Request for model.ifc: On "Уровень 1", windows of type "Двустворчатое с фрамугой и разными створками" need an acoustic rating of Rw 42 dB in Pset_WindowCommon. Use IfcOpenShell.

First a look at what the model holds.

```python
import ifcopenshell
import ifcopenshell.util.element

model = ifcopenshell.open("model.ifc")
print(model.schema)
storey = next(s for s in model.by_type("IfcBuildingStorey") if s.Name == "Уровень 1")
windows = [e for e in ifcopenshell.util.element.get_decomposition(storey) if e.is_a("IfcWindow")]
seen = {}
for e in windows:
    element_type = ifcopenshell.util.element.get_type(e)
    key = (element_type.Name if element_type != e and element_type else None, ifcopenshell.util.element.get_pset(e, "Pset_WindowCommon", "AcousticRating"))
    seen[key] = seen.get(key, 0) + 1
for (name, value), count in sorted(seen.items(), key=str):
    print(count, "x", name, "|", value)
```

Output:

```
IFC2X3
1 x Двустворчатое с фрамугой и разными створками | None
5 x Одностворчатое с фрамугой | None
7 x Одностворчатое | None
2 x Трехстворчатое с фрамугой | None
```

```python
import ifcopenshell
import ifcopenshell.api.pset
import ifcopenshell.util.element

model = ifcopenshell.open("model.ifc")

storey = next(s for s in model.by_type("IfcBuildingStorey") if s.Name == "Уровень 1")
windows = [e for e in ifcopenshell.util.element.get_decomposition(storey) if e.is_a("IfcWindow")]

count = 0
for e in windows:
    element_type = ifcopenshell.util.element.get_type(e)
    if element_type in (None, e) or element_type.Name != "Двустворчатое с фрамугой и разными створками":
        continue
    # add_pset returns the element's existing set when there is one.
    pset = ifcopenshell.api.pset.add_pset(model, product=e, name="Pset_WindowCommon")
    ifcopenshell.api.pset.edit_pset(model, pset=pset, properties={"AcousticRating": "Rw 42 dB"})
    count += 1

print(count, "windows updated")

model.write("model_edited.ifc")
```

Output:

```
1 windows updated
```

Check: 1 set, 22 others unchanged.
